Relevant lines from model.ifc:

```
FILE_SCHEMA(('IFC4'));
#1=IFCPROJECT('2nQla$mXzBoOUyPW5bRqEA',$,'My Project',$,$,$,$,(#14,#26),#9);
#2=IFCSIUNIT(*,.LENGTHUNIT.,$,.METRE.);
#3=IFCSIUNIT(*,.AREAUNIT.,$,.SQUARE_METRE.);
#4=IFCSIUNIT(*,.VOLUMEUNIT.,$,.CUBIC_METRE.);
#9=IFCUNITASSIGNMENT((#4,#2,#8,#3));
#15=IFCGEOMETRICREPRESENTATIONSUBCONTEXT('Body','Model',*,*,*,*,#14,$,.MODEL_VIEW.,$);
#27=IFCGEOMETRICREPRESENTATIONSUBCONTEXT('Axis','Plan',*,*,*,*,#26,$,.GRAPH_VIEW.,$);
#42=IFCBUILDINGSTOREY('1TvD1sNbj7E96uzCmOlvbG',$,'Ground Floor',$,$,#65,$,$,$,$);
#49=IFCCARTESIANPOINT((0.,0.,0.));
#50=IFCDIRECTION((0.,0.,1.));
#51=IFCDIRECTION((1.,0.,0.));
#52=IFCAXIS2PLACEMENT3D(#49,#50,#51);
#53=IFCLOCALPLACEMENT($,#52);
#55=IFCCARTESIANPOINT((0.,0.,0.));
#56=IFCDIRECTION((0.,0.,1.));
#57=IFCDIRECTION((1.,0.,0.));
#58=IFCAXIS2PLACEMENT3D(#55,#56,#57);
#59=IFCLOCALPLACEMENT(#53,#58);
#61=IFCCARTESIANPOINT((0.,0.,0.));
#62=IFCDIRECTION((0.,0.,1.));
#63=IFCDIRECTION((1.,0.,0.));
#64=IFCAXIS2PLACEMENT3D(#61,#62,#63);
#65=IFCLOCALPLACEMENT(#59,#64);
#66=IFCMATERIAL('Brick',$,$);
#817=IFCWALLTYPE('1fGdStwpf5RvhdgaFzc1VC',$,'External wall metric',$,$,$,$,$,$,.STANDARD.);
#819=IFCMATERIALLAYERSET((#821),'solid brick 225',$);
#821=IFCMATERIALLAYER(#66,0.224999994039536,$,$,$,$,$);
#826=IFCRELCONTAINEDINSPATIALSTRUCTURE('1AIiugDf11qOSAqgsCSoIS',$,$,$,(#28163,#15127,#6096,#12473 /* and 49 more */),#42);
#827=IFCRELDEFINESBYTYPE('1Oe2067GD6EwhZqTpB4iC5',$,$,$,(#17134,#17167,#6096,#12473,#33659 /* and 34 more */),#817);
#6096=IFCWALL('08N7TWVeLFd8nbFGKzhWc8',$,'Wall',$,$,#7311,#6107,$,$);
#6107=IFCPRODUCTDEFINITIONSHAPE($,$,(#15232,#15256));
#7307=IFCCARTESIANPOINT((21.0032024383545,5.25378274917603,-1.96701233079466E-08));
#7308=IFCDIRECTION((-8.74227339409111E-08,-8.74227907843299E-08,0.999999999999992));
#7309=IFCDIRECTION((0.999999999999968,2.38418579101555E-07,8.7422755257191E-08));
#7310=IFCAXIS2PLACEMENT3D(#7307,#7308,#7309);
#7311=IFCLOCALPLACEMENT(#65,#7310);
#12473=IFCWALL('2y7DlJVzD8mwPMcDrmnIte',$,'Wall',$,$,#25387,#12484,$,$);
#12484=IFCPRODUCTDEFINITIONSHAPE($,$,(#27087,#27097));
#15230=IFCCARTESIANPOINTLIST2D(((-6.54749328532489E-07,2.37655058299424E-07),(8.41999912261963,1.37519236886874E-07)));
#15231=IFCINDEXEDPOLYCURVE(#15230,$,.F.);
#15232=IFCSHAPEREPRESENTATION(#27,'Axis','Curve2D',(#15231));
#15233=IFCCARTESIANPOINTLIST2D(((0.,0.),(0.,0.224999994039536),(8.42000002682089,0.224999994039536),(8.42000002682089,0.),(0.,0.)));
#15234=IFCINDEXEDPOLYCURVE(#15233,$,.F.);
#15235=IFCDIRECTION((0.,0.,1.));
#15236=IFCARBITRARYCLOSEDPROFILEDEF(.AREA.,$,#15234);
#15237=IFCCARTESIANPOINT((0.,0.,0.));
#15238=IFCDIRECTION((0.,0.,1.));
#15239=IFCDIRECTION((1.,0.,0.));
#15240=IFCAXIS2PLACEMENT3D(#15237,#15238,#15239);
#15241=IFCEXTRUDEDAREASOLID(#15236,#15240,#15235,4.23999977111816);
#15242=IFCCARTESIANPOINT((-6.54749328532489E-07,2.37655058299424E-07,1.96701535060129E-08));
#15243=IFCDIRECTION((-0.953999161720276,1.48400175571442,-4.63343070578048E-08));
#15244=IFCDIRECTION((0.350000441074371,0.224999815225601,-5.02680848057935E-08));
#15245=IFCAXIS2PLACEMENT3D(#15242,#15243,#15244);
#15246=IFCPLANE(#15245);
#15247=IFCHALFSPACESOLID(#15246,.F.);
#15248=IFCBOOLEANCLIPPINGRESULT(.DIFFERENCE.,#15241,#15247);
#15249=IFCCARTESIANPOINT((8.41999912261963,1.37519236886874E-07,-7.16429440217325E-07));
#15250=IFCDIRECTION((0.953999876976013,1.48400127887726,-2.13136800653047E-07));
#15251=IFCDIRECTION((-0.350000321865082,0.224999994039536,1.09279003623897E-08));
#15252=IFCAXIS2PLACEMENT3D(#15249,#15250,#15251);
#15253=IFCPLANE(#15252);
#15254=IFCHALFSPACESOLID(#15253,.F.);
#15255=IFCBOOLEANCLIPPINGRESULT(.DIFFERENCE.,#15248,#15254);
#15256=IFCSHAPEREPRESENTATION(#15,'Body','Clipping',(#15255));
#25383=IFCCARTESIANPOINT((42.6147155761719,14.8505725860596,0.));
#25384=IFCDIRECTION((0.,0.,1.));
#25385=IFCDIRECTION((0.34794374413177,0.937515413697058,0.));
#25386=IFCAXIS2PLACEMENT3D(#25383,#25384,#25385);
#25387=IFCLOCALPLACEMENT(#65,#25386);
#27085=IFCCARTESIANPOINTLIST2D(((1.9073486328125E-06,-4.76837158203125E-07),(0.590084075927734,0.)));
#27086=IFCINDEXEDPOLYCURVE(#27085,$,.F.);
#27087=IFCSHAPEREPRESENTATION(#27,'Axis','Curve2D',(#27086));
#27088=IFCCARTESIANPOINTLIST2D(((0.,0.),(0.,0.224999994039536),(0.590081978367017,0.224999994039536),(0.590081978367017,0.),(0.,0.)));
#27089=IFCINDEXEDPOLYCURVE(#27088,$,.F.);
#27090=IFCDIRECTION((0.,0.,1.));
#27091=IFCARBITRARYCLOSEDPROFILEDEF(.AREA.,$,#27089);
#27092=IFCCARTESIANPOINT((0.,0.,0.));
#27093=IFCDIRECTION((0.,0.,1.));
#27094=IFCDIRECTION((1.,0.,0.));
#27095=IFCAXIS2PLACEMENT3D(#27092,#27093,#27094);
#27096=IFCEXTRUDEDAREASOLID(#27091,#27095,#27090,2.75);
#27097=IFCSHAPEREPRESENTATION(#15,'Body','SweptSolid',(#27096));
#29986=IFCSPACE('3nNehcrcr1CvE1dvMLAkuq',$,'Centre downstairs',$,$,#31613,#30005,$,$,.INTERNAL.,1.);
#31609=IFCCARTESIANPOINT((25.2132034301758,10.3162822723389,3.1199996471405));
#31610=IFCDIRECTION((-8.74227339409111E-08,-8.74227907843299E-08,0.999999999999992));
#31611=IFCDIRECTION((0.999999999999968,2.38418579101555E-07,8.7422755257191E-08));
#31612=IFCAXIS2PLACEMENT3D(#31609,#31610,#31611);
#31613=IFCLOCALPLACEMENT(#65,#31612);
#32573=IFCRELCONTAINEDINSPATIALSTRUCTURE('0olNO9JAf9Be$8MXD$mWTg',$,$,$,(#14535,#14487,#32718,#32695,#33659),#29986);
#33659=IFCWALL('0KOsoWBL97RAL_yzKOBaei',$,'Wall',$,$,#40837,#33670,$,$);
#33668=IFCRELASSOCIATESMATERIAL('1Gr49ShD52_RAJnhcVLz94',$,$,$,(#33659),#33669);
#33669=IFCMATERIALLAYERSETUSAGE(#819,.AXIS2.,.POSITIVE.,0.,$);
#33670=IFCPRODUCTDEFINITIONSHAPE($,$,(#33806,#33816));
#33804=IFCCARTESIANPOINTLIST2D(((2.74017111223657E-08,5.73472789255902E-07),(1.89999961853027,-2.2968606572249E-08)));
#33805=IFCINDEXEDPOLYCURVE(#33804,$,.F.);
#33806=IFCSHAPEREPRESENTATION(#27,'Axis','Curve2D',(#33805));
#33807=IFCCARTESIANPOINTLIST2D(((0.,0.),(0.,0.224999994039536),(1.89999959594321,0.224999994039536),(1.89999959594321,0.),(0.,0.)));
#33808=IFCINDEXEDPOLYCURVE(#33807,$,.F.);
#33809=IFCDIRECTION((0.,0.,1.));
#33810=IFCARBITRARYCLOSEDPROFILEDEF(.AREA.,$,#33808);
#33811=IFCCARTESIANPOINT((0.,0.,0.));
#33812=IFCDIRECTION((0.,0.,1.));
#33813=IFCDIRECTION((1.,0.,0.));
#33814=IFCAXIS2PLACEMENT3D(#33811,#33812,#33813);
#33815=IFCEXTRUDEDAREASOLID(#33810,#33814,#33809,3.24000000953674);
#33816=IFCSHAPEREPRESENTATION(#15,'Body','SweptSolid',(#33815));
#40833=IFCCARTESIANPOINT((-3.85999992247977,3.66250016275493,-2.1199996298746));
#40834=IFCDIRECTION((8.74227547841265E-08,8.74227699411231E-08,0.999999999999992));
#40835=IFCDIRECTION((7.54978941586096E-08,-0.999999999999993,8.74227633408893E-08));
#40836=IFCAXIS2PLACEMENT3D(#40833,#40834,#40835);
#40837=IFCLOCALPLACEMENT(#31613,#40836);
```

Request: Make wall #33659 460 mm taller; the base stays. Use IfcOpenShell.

```python
import ifcopenshell
import ifcopenshell.geom
import ifcopenshell.util.representation
import ifcopenshell.util.shape

model = ifcopenshell.open("model.ifc")
settings = ifcopenshell.geom.settings()


def volume(element):
    """Net volume in cubic metres, openings subtracted."""
    shape = ifcopenshell.geom.create_shape(settings, element)
    return ifcopenshell.util.shape.get_volume(shape.geometry)


wall = model.by_id(33659)
before = volume(wall)

body = ifcopenshell.util.representation.get_representation(wall, "Model", "Body")
solid = body.Items[0]
old_height = solid.Depth
solid.Depth += 0.46
after = volume(wall)

print(f"height {old_height:g} -> {solid.Depth:g}, volume {before:.3f} -> {after:.3f} m3")

model.write("model_v2.ifc")
```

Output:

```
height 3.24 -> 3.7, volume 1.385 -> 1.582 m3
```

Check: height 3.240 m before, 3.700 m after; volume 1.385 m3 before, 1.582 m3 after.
